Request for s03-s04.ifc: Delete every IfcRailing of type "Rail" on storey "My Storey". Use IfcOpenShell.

First a look at what the model holds.

```python
import ifcopenshell
import ifcopenshell.util.element

model = ifcopenshell.open("s03-s04.ifc")
print(model.schema)
storey = next(s for s in model.by_type("IfcBuildingStorey") if s.Name == "My Storey")
railings = [e for e in ifcopenshell.util.element.get_decomposition(storey) if e.is_a("IfcRailing")]
seen = {}
for e in railings:
    element_type = ifcopenshell.util.element.get_type(e)
    name = element_type.Name if element_type not in (None, e) else None
    seen[name] = seen.get(name, 0) + 1
for name, count in sorted(seen.items(), key=str):
    print(count, "x", name)
```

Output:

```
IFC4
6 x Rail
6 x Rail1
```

```python
import ifcopenshell
import ifcopenshell.api.root
import ifcopenshell.util.element

model = ifcopenshell.open("s03-s04.ifc")

storey = next(s for s in model.by_type("IfcBuildingStorey") if s.Name == "My Storey")
railings = [e for e in ifcopenshell.util.element.get_decomposition(storey) if e.is_a("IfcRailing")]
targets = [e for e in railings if (t := ifcopenshell.util.element.get_type(e)) not in (None, e) and t.Name == "Rail"]

for e in targets:
    ifcopenshell.api.root.remove_product(model, product=e)
print(len(targets), "removed")

model.write("s03-s04_edited.ifc")
```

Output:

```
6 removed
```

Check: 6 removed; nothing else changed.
